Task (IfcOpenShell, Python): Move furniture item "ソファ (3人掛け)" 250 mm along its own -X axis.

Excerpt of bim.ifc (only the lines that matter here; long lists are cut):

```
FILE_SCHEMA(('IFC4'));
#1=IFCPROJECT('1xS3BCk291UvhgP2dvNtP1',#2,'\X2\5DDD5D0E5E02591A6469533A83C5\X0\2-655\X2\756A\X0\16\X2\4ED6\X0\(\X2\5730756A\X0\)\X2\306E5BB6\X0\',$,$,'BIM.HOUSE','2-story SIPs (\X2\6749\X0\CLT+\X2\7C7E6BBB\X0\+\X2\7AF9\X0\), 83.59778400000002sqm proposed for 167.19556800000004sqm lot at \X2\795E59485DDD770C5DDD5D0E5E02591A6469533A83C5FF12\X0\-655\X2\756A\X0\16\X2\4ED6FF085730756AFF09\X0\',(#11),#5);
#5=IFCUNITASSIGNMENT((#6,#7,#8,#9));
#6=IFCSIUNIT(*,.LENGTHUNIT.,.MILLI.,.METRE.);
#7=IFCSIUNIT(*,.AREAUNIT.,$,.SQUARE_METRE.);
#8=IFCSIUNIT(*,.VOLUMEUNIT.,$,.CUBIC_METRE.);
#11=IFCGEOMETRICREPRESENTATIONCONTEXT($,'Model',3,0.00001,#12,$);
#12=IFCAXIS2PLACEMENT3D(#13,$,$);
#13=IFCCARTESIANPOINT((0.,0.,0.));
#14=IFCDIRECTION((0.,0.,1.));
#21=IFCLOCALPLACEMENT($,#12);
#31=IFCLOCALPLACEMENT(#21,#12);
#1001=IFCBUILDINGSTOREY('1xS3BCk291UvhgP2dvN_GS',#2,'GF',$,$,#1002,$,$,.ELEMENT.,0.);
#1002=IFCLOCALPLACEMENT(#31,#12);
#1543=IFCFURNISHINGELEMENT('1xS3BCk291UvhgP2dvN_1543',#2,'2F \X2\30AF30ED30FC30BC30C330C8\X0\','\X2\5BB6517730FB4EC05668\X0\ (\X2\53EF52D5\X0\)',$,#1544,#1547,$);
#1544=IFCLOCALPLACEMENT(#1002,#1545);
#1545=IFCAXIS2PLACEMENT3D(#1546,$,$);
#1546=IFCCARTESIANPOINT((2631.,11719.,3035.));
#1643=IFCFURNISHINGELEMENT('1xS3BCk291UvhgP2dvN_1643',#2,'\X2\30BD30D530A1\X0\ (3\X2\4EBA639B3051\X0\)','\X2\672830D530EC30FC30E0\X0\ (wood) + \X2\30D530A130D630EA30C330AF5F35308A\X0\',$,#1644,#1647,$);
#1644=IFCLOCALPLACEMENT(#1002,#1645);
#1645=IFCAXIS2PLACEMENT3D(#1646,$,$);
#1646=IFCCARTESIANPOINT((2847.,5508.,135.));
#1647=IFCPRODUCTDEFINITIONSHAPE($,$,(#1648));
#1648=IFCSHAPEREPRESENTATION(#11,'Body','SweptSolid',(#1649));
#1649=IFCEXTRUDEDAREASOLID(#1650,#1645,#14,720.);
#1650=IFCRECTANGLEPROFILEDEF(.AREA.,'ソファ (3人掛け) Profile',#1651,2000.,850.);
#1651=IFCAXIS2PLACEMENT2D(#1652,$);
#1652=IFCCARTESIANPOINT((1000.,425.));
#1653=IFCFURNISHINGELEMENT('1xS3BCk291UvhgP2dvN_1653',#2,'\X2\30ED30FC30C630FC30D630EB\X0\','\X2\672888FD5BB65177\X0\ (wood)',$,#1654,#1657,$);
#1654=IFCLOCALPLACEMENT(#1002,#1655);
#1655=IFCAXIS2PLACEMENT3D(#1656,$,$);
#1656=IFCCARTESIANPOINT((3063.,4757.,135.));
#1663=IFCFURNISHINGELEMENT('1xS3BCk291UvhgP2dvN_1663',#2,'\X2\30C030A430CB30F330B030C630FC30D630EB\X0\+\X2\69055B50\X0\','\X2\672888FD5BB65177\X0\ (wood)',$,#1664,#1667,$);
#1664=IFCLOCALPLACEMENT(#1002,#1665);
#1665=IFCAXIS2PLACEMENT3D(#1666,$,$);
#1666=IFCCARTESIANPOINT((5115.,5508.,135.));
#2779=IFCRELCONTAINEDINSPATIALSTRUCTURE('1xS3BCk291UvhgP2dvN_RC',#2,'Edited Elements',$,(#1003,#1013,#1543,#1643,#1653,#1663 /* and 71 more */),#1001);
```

```python
import ifcopenshell
import ifcopenshell.api.geometry
import ifcopenshell.util.placement

model = ifcopenshell.open("bim.ifc")

item = model.by_id(1643)
matrix = ifcopenshell.util.placement.get_local_placement(item.ObjectPlacement)
matrix[:3, 3] -= matrix[:3, 0] * 250.0
ifcopenshell.api.geometry.edit_object_placement(model, product=item, matrix=matrix, is_si=False)

print(ifcopenshell.util.placement.get_local_placement(item.ObjectPlacement).round(3) + 0.0)

model.write("bim_rev.ifc")
```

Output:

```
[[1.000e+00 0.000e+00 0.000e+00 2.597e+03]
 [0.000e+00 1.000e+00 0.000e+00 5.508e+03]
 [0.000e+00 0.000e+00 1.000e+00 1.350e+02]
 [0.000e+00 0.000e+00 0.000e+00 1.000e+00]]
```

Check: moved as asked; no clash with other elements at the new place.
